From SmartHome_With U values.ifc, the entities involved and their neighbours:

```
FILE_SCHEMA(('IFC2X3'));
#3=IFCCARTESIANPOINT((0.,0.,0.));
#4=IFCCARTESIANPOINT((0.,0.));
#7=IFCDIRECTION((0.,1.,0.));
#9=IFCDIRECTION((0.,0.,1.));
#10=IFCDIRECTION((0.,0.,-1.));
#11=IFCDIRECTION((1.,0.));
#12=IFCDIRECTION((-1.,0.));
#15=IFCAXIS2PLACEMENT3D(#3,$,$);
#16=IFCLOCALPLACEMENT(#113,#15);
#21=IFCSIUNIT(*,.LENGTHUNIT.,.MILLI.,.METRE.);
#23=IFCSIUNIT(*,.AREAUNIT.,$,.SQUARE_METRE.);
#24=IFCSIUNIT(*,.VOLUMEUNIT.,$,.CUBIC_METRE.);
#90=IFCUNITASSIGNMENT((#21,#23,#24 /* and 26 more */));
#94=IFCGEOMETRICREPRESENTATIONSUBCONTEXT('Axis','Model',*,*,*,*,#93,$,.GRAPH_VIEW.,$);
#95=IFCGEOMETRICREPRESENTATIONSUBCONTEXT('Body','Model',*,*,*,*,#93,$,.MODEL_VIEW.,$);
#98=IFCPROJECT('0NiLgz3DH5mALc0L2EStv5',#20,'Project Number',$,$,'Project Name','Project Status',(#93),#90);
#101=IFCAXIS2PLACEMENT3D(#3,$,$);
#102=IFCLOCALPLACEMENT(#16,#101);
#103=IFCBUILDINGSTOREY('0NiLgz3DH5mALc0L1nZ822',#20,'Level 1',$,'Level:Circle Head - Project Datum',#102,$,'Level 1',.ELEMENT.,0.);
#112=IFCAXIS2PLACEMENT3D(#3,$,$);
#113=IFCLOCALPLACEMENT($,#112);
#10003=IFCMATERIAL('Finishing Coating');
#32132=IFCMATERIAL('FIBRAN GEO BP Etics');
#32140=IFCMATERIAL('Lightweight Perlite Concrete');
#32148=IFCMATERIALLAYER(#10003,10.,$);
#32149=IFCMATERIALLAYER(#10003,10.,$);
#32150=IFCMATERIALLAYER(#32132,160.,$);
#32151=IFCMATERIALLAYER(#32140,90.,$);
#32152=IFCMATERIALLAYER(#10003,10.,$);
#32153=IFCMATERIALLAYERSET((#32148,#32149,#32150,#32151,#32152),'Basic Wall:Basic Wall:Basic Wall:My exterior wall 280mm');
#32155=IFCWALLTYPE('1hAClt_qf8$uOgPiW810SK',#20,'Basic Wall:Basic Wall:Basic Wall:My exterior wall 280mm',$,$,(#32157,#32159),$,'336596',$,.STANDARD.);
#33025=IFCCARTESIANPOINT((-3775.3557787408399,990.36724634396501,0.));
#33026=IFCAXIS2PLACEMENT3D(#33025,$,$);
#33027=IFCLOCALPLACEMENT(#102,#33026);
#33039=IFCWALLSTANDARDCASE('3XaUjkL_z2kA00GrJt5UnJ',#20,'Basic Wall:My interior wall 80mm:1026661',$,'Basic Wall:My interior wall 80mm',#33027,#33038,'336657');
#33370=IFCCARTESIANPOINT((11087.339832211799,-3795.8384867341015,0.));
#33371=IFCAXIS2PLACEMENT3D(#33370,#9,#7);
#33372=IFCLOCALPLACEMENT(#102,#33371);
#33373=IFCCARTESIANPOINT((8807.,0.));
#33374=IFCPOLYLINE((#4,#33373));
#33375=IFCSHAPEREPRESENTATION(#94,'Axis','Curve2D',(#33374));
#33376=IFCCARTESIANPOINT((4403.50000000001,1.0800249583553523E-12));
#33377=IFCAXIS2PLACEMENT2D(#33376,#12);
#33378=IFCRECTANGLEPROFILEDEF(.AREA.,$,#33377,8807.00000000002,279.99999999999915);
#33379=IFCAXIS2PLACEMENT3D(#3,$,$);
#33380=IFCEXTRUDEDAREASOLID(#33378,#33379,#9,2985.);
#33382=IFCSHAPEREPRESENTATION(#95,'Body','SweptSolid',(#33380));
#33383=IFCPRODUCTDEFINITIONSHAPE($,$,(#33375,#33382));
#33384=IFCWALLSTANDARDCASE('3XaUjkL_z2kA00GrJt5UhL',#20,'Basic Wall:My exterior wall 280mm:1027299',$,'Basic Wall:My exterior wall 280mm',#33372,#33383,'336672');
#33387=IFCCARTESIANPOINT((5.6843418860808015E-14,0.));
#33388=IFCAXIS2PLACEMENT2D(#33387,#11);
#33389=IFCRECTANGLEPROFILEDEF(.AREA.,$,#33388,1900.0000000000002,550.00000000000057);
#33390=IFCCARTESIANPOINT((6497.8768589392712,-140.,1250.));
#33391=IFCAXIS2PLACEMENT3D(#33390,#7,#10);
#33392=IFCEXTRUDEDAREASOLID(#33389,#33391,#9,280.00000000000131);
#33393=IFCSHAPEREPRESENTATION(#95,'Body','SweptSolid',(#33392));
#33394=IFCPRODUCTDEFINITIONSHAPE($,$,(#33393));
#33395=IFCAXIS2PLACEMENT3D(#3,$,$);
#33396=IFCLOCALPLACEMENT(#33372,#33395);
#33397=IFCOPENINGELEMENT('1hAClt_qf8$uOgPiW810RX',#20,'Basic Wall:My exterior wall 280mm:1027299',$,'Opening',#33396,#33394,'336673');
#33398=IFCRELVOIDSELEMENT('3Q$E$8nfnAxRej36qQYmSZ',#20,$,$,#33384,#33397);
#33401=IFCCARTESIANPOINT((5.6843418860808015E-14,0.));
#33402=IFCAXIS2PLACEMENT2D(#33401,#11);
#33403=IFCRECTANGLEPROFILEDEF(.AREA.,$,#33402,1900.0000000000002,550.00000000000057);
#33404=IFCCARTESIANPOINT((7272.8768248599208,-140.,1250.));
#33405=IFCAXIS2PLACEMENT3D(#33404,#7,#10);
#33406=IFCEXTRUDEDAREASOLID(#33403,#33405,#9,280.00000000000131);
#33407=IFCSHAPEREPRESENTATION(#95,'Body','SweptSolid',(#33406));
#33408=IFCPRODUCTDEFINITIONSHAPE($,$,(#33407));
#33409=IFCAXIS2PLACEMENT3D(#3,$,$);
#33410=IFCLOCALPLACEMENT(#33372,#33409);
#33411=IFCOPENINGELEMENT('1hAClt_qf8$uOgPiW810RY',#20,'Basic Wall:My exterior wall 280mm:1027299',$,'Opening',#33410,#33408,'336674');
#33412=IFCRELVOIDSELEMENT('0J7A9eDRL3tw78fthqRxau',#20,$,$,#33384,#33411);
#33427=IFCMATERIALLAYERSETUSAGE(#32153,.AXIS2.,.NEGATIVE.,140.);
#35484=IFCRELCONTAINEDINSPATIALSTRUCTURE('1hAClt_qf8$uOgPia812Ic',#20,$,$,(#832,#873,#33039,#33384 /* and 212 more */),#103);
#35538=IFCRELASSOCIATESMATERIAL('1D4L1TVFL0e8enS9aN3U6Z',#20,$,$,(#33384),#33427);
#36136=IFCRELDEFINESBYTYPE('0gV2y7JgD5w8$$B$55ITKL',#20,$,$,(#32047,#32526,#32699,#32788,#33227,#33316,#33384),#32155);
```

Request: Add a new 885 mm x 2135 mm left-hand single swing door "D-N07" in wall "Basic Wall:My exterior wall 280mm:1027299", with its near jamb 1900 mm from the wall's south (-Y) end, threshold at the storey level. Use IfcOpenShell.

```python
import numpy as np
import ifcopenshell
import ifcopenshell.api.feature
import ifcopenshell.api.geometry
import ifcopenshell.api.root
import ifcopenshell.api.spatial
import ifcopenshell.api.type
import ifcopenshell.geom
import ifcopenshell.util.element
import ifcopenshell.util.placement
import ifcopenshell.util.representation
import ifcopenshell.util.shape
import ifcopenshell.util.unit

model = ifcopenshell.open("SmartHome_With U values.ifc")
unit_scale = ifcopenshell.util.unit.calculate_unit_scale(model)
settings = ifcopenshell.geom.settings()


def volume(element):
    """Net volume in cubic metres, openings subtracted."""
    shape = ifcopenshell.geom.create_shape(settings, element)
    return ifcopenshell.util.shape.get_volume(shape.geometry)


wall = model.by_guid("3XaUjkL_z2kA00GrJt5UhL")
storey = ifcopenshell.util.element.get_container(wall, ifc_class="IfcBuildingStorey")
context = ifcopenshell.util.representation.get_context(model, "Model", "Body", "MODEL_VIEW")
before = volume(wall)

width, height, from_end, sill = 0.885, 2.135, 1.9, 0.0  # metres

# The wall runs along its own X axis, and the end named is its -X end.
wall_shape = ifcopenshell.geom.create_shape(settings, wall)
x, y, z = ifcopenshell.util.shape.get_vertices(wall_shape.geometry).T
start = x.min() + from_end
face, thickness = float(y.min()), float(y.max() - y.min())
wall_matrix = ifcopenshell.util.placement.get_local_placement(wall.ObjectPlacement)
level = ifcopenshell.util.placement.get_local_placement(storey.ObjectPlacement)[2, 3]


def in_wall(x, y):
    """Placement at x, y metres in the wall's axes, at sill height."""
    matrix = wall_matrix.copy()
    matrix[:, 3] = wall_matrix @ np.array([x / unit_scale, y / unit_scale, 0.0, 1.0])
    matrix[2, 3] = level + sill / unit_scale
    return matrix


# Opening: a box that overshoots both wall faces by 50 mm.
opening = ifcopenshell.api.root.create_entity(model, ifc_class="IfcOpeningElement")
box = ifcopenshell.api.geometry.add_wall_representation(
    model, context=context, length=width, height=height, thickness=thickness + 0.1
)
ifcopenshell.api.geometry.assign_representation(model, product=opening, representation=box)
ifcopenshell.api.geometry.edit_object_placement(model, product=opening, matrix=in_wall(start, face - 0.05), is_si=False)
ifcopenshell.api.feature.add_feature(model, feature=opening, element=wall)

door = ifcopenshell.api.root.create_entity(model, ifc_class="IfcDoor", name="D-N07")
door.OverallWidth, door.OverallHeight = width / unit_scale, height / unit_scale
body = ifcopenshell.api.geometry.add_door_representation(
    model,
    context=context,
    overall_width=door.OverallWidth,
    overall_height=door.OverallHeight,
    operation_type="SINGLE_SWING_LEFT",
    lining_properties={"LiningDepth": thickness / unit_scale, "ThresholdDepth": thickness / unit_scale},
)
ifcopenshell.api.geometry.assign_representation(model, product=door, representation=body)
ifcopenshell.api.spatial.assign_container(model, products=[door], relating_structure=storey)
fills = ifcopenshell.api.feature.add_filling(model, opening=opening, element=door)
fills.OwnerHistory = door.OwnerHistory  # required in IFC2X3

# IFC2X3 keeps the operation on the door style.
style = ifcopenshell.api.root.create_entity(model, ifc_class="IfcDoorStyle", name="D-N07")
style.OperationType, style.ConstructionType = "SINGLE_SWING_LEFT", "NOTDEFINED"
style.ParameterTakesPrecedence = style.Sizeable = False
ifcopenshell.api.type.assign_type(model, related_objects=[door], relating_type=style)

# The lining spans the wall, so the door starts at the wall face.
ifcopenshell.api.geometry.edit_object_placement(model, product=door, matrix=in_wall(start, face), is_si=False)

after = volume(wall)

print(f"wall volume {before:.3f} -> {after:.3f} m3")

model.write("SmartHome_With U values-out.ifc")
```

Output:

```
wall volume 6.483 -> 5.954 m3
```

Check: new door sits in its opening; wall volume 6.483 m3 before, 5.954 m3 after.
